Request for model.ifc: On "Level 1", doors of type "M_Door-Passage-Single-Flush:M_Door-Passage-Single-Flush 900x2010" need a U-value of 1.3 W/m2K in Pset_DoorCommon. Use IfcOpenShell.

First a look at what the model holds.

```python
import ifcopenshell
import ifcopenshell.util.element

model = ifcopenshell.open("model.ifc")
print(model.schema)
storey = next(s for s in model.by_type("IfcBuildingStorey") if s.Name == "Level 1")
doors = [e for e in ifcopenshell.util.element.get_decomposition(storey) if e.is_a("IfcDoor")]
seen = {}
for e in doors:
    element_type = ifcopenshell.util.element.get_type(e)
    key = (element_type.Name if element_type != e and element_type else None, ifcopenshell.util.element.get_pset(e, "Pset_DoorCommon", "ThermalTransmittance"))
    seen[key] = seen.get(key, 0) + 1
for (name, value), count in sorted(seen.items(), key=str):
    print(count, "x", name, "|", value)
```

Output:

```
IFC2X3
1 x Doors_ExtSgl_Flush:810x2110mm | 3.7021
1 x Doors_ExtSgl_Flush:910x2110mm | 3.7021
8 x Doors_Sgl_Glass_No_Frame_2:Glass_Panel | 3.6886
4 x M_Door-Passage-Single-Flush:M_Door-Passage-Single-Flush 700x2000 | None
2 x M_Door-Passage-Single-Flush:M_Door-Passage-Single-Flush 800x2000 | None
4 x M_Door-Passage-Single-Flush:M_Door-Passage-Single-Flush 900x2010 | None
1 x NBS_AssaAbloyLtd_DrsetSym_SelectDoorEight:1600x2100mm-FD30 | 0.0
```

```python
import ifcopenshell
import ifcopenshell.api.pset
import ifcopenshell.util.element

model = ifcopenshell.open("model.ifc")

storey = next(s for s in model.by_type("IfcBuildingStorey") if s.Name == "Level 1")
doors = [e for e in ifcopenshell.util.element.get_decomposition(storey) if e.is_a("IfcDoor")]

count = 0
for e in doors:
    element_type = ifcopenshell.util.element.get_type(e)
    if element_type in (None, e) or element_type.Name != "M_Door-Passage-Single-Flush:M_Door-Passage-Single-Flush 900x2010":
        continue
    # add_pset returns the element's existing set when there is one.
    pset = ifcopenshell.api.pset.add_pset(model, product=e, name="Pset_DoorCommon")
    ifcopenshell.api.pset.edit_pset(model, pset=pset, properties={"ThermalTransmittance": 1.3})
    count += 1

print(count, "doors updated")

model.write("model_updated.ifc")
```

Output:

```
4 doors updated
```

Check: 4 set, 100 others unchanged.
